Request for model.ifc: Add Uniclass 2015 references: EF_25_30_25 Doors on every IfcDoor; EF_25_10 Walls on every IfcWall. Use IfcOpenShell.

First a look at what the model holds.

```python
import ifcopenshell

model = ifcopenshell.open("model.ifc")
print(model.schema)
print("classifications:", [c.Name for c in model.by_type("IfcClassification")])
for ifc_class in ("IfcDoor", "IfcRoof", "IfcStair", "IfcWall", "IfcWindow"):
    print(ifc_class, len(model.by_type(ifc_class)))
```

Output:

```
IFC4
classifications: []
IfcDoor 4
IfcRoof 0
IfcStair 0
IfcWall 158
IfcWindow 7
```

```python
import ifcopenshell
import ifcopenshell.api.classification

model = ifcopenshell.open("model.ifc")

system = ifcopenshell.api.classification.add_classification(model, classification="Uniclass 2015")

codes = {
    "IfcDoor": ("EF_25_30_25", "Doors"),
    "IfcWall": ("EF_25_10", "Walls"),
}
for ifc_class, (code, name) in codes.items():
    products = model.by_type(ifc_class)
    ifcopenshell.api.classification.add_reference(
        model, products=products, classification=system, identification=code, name=name
    )
    print(code, len(products))

model.write("model_v2.ifc")
```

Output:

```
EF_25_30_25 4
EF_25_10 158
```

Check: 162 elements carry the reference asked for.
